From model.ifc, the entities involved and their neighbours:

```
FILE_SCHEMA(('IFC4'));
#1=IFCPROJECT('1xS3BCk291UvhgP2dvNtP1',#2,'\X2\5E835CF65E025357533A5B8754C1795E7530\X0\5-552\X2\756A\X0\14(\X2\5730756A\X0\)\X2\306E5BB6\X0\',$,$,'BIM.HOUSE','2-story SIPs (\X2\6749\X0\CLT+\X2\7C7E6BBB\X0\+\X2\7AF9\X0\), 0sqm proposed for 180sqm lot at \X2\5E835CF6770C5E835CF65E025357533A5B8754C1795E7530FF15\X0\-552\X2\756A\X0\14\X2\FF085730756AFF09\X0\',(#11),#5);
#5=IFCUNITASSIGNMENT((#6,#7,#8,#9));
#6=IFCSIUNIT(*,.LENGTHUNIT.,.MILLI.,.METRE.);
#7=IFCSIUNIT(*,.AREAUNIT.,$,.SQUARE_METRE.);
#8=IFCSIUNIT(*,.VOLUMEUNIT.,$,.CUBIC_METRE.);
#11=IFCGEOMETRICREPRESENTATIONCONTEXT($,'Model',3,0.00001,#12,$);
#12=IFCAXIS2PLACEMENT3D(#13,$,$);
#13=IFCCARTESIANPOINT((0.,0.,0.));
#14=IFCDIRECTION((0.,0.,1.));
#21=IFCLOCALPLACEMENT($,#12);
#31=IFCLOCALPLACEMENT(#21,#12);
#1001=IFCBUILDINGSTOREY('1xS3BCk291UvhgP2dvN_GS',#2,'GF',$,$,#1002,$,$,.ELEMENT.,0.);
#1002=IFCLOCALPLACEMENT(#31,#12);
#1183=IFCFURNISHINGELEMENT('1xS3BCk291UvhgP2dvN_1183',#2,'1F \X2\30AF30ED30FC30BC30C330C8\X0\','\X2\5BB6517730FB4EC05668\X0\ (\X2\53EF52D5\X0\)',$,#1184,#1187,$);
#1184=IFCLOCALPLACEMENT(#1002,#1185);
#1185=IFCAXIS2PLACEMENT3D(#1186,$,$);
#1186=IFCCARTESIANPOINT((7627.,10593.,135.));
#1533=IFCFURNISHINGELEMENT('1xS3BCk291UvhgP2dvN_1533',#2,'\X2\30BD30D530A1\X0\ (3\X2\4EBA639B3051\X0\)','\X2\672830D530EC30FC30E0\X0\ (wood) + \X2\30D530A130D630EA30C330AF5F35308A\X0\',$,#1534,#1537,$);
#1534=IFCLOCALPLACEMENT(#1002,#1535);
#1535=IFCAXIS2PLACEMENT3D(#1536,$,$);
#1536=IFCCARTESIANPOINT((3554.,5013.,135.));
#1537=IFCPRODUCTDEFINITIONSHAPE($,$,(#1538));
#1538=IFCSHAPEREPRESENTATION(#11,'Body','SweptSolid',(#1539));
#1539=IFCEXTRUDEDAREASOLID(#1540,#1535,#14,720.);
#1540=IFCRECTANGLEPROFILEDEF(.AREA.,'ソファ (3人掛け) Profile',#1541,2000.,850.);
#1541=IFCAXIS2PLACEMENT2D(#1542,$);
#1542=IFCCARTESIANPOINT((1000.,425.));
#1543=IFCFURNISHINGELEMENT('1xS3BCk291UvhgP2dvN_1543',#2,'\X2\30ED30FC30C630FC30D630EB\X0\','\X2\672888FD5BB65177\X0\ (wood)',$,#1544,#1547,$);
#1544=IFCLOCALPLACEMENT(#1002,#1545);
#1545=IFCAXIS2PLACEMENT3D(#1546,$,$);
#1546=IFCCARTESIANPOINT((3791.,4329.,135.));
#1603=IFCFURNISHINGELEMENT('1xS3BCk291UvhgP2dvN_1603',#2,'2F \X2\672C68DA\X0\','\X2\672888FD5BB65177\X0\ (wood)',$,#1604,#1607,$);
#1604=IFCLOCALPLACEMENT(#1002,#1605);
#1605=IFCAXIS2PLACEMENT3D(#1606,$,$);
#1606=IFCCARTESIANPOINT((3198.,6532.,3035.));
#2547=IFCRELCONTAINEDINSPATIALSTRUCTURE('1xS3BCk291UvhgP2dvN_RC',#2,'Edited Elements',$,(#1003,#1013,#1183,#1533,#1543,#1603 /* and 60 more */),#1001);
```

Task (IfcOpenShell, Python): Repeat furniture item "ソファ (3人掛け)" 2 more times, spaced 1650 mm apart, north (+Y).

```python
import numpy as np
import ifcopenshell
import ifcopenshell.api.geometry
import ifcopenshell.api.root
import ifcopenshell.util.element
import ifcopenshell.util.placement
import ifcopenshell.util.unit

model = ifcopenshell.open("model.ifc")
unit_scale = ifcopenshell.util.unit.calculate_unit_scale(model)


def reuse_history(source, copy):
    """copy_class also copies each property set's owner history, people and application; keep the originals."""
    for rel in copy.IsDefinedBy:
        if rel.is_a("IfcRelDefinesByProperties") and (history := rel.RelatingPropertyDefinition.OwnerHistory):
            rel.RelatingPropertyDefinition.OwnerHistory = source.OwnerHistory
            ifcopenshell.util.element.remove_deep2(model, history)


source = model.by_guid("1xS3BCk291UvhgP2dvN_1533")
base = ifcopenshell.util.placement.get_local_placement(source.ObjectPlacement)
step = np.array([0.0, 1.0, 0.0]) * 1.65 / unit_scale

for i in range(1, 3):
    copy = ifcopenshell.api.root.copy_class(model, product=source)
    copy.Representation = ifcopenshell.util.element.copy_deep(
        model, source.Representation, exclude=["IfcGeometricRepresentationContext", "IfcRepresentationMap"]
    )
    reuse_history(source, copy)
    matrix = base.copy()
    matrix[:3, 3] += i * step
    print("added at", matrix[:3, 3].round(3) + 0.0)
    ifcopenshell.api.geometry.edit_object_placement(model, product=copy, matrix=matrix, is_si=False)

model.write("model-out.ifc")
```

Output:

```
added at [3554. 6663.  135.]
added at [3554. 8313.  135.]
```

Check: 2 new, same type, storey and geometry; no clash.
